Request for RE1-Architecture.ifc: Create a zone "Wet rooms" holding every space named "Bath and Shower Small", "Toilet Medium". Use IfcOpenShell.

First a look at what the model holds.

```python
import ifcopenshell

model = ifcopenshell.open("RE1-Architecture.ifc")
print(model.schema)
seen = {}
for space in model.by_type("IfcSpace"):
    seen[space.LongName] = seen.get(space.LongName, 0) + 1
for name, count in sorted(seen.items(), key=str):
    print(count, "x", name)
print("zones:", [z.Name for z in model.by_type("IfcZone")][:20])
```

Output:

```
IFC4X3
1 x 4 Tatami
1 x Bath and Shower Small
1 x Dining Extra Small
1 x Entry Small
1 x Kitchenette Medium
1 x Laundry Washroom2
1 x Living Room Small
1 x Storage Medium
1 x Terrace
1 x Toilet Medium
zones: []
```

```python
import ifcopenshell
import ifcopenshell.api.group
import ifcopenshell.api.root

model = ifcopenshell.open("RE1-Architecture.ifc")

names = {"Bath and Shower Small", "Toilet Medium"}
spaces = [s for s in model.by_type("IfcSpace") if s.LongName in names]

zone = ifcopenshell.api.root.create_entity(model, ifc_class="IfcZone", name="Wet rooms")
ifcopenshell.api.group.assign_group(model, products=spaces, group=zone)
print(len(spaces), "spaces in", zone.Name)

model.write("RE1-Architecture_edited.ifc")
```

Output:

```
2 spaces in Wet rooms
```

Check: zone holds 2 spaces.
